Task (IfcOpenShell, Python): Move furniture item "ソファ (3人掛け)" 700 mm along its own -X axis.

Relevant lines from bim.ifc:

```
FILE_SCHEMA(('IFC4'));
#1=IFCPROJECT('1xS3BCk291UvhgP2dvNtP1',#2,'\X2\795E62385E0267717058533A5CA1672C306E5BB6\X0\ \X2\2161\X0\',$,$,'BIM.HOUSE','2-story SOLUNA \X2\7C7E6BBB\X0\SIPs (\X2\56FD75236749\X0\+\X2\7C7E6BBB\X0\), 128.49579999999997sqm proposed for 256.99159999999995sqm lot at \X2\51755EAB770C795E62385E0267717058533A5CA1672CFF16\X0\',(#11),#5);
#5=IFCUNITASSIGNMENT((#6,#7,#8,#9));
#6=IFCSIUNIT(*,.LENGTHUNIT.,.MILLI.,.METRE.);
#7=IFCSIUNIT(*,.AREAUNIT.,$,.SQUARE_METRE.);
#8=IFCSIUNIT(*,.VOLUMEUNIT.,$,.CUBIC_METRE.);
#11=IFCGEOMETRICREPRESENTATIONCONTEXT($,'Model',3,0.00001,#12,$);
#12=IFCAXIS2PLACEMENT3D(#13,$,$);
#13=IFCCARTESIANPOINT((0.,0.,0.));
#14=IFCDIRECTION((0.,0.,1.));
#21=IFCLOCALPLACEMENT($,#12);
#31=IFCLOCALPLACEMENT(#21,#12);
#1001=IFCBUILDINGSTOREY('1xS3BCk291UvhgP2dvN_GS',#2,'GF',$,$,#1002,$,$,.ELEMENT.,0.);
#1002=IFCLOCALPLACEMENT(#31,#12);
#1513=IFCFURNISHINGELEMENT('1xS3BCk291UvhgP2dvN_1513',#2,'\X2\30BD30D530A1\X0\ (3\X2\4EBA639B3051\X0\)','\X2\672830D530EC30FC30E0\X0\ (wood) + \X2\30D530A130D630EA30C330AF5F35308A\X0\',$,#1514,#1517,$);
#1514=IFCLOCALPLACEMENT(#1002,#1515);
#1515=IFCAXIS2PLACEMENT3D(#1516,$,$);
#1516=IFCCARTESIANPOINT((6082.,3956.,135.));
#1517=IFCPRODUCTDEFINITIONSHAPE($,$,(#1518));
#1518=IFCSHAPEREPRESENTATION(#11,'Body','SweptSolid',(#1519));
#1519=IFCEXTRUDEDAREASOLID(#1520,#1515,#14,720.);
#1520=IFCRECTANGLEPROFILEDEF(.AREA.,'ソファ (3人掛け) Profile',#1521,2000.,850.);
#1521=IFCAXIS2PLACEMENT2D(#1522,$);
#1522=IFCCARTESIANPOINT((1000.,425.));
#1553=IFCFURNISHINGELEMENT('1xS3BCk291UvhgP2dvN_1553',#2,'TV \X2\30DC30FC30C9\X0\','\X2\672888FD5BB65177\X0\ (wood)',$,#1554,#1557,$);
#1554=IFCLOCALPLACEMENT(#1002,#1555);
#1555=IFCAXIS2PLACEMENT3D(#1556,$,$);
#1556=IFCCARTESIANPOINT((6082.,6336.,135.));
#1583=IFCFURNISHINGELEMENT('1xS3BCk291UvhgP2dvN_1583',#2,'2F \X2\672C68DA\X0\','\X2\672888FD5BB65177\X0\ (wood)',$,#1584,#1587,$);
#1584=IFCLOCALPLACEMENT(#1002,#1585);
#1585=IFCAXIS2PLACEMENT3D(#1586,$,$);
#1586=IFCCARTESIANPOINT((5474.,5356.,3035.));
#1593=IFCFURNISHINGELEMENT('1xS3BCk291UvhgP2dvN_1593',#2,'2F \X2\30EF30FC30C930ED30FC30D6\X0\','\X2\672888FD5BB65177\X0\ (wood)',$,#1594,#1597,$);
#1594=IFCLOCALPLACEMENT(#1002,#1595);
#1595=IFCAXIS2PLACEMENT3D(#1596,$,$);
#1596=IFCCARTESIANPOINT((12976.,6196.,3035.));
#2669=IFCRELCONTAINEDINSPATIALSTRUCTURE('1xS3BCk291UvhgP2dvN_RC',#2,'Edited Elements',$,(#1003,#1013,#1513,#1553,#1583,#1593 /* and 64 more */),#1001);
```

```python
import ifcopenshell
import ifcopenshell.api.geometry
import ifcopenshell.util.placement
import ifcopenshell.util.unit

model = ifcopenshell.open("bim.ifc")
unit_scale = ifcopenshell.util.unit.calculate_unit_scale(model)

item = model.by_id(1513)
matrix = ifcopenshell.util.placement.get_local_placement(item.ObjectPlacement)
matrix[:3, 3] -= matrix[:3, 0] * 0.7 / unit_scale
ifcopenshell.api.geometry.edit_object_placement(model, product=item, matrix=matrix, is_si=False)

print(ifcopenshell.util.placement.get_local_placement(item.ObjectPlacement).round(3) + 0.0)

model.write("bim-out.ifc")
```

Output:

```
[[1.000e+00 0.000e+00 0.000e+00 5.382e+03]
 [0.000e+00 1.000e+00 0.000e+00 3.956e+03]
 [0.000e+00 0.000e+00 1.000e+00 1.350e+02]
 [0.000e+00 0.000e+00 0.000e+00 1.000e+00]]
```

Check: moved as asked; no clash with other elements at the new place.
